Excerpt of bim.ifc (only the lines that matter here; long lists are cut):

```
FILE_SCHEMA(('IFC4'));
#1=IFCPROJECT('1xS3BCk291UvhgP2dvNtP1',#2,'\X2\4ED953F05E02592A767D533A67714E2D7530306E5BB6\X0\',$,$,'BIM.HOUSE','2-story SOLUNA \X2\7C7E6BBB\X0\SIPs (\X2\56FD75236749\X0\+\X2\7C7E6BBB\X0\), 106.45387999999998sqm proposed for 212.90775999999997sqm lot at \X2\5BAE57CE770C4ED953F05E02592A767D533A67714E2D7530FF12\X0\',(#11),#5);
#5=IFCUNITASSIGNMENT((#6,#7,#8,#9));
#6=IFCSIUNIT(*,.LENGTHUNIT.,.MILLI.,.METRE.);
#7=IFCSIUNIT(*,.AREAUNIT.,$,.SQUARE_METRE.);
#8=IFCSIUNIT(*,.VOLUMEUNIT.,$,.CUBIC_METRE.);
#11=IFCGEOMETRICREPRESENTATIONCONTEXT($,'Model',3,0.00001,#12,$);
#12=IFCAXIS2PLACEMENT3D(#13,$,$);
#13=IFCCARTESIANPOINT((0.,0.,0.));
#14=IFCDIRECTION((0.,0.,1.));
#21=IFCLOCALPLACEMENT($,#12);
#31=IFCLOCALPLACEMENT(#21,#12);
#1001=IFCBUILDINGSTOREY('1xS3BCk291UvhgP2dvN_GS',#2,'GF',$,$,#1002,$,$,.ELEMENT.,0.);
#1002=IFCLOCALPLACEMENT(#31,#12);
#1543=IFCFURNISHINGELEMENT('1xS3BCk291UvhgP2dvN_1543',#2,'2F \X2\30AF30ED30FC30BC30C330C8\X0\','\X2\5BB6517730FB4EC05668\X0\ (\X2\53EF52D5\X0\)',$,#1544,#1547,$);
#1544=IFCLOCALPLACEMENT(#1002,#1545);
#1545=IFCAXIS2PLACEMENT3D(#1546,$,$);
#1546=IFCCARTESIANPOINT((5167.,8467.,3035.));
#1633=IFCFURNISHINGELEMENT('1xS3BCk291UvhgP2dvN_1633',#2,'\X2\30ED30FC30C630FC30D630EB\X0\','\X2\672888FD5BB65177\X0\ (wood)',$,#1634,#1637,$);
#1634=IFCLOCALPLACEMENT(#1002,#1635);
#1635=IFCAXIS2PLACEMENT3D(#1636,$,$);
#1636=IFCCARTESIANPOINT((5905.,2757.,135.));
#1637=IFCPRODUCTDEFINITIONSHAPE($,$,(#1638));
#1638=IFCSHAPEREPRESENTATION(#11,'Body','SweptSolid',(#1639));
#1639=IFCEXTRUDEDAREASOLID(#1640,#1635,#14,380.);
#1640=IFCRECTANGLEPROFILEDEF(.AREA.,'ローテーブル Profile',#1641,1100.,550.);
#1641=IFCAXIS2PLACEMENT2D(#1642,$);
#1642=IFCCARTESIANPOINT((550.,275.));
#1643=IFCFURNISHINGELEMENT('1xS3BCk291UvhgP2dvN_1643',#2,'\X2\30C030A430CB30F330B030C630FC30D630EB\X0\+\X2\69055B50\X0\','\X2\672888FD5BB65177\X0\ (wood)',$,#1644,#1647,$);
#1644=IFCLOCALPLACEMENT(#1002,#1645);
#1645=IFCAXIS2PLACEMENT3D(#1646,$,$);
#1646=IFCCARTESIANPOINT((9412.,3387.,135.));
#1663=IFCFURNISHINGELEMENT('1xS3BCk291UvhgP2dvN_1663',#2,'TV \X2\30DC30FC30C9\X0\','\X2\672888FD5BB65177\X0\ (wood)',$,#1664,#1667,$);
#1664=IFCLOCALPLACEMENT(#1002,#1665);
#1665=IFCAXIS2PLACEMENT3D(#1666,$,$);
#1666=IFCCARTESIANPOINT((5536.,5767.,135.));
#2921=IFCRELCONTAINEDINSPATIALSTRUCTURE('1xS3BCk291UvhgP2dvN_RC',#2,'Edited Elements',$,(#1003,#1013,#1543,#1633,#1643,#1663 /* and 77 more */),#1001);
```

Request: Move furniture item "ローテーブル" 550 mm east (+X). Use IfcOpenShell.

```python
import ifcopenshell
import ifcopenshell.api.geometry
import ifcopenshell.util.placement
import ifcopenshell.util.unit

model = ifcopenshell.open("bim.ifc")
unit_scale = ifcopenshell.util.unit.calculate_unit_scale(model)

item = model.by_id(1633)
matrix = ifcopenshell.util.placement.get_local_placement(item.ObjectPlacement)
matrix[0, 3] += 0.55 / unit_scale
ifcopenshell.api.geometry.edit_object_placement(model, product=item, matrix=matrix, is_si=False)

print(ifcopenshell.util.placement.get_local_placement(item.ObjectPlacement).round(3) + 0.0)

model.write("bim_v2.ifc")
```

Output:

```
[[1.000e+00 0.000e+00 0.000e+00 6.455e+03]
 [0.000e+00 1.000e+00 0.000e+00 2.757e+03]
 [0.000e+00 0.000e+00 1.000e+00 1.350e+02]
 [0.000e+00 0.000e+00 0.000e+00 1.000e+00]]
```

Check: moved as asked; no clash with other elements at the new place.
